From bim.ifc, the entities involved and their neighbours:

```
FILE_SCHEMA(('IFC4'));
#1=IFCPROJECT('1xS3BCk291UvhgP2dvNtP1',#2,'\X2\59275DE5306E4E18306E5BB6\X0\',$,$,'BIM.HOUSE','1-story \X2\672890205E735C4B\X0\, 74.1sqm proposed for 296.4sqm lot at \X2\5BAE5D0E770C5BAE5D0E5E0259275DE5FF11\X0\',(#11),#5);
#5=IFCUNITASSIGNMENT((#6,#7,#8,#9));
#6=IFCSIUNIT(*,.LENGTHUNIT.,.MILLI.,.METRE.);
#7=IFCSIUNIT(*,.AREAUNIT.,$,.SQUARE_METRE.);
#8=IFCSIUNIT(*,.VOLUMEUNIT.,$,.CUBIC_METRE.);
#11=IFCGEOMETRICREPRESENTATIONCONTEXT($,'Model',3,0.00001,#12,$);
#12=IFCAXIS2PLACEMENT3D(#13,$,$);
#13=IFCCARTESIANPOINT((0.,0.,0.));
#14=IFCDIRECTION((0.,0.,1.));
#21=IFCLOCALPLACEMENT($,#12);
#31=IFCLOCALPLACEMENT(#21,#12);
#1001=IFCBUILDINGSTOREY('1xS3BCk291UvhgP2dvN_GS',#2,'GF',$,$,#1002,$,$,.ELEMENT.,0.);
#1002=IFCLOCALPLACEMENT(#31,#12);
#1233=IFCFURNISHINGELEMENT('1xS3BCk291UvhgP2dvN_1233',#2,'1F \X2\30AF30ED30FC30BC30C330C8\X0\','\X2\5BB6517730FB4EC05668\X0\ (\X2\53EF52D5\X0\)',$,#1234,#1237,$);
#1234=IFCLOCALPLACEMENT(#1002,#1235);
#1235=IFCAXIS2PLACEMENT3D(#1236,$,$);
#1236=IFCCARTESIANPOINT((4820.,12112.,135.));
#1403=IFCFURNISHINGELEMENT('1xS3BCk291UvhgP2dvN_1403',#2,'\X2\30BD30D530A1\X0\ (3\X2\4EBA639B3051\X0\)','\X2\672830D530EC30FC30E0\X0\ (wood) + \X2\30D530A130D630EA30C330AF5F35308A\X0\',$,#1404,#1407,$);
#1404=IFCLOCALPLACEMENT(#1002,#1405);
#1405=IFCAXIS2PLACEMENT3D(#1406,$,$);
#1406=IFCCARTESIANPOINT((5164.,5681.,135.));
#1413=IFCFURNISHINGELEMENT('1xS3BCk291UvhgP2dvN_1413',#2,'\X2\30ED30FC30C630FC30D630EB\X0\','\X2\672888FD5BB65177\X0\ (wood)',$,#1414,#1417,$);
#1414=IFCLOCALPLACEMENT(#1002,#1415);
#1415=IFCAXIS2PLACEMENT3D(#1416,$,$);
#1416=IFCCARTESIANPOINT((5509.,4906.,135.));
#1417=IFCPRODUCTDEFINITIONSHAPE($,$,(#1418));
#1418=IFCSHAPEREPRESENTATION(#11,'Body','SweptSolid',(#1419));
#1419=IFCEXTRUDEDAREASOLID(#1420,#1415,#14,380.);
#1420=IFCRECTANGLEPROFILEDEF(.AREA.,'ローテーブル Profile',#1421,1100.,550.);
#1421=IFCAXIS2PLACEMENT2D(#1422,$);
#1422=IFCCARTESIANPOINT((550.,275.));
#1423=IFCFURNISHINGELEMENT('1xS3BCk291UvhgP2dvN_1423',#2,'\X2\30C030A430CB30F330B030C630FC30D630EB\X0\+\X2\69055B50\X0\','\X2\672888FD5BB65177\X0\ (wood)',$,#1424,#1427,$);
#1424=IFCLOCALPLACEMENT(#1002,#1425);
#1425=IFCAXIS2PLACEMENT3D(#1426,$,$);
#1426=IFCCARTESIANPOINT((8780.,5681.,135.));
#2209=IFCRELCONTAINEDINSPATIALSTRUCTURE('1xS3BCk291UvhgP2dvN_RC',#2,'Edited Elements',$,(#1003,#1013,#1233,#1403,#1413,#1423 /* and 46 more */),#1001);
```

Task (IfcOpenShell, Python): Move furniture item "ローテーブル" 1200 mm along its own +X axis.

```python
import ifcopenshell
import ifcopenshell.api.geometry
import ifcopenshell.util.placement
import ifcopenshell.util.unit

model = ifcopenshell.open("bim.ifc")
unit_scale = ifcopenshell.util.unit.calculate_unit_scale(model)

item = model.by_guid("1xS3BCk291UvhgP2dvN_1413")
matrix = ifcopenshell.util.placement.get_local_placement(item.ObjectPlacement)
matrix[:3, 3] += matrix[:3, 0] * 1.2 / unit_scale
ifcopenshell.api.geometry.edit_object_placement(model, product=item, matrix=matrix, is_si=False)

print(ifcopenshell.util.placement.get_local_placement(item.ObjectPlacement).round(3) + 0.0)

model.write("bim-out.ifc")
```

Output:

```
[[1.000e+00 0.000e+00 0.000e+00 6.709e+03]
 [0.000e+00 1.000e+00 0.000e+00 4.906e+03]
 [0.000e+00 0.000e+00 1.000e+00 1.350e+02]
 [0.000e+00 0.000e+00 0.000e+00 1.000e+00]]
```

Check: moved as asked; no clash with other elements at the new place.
